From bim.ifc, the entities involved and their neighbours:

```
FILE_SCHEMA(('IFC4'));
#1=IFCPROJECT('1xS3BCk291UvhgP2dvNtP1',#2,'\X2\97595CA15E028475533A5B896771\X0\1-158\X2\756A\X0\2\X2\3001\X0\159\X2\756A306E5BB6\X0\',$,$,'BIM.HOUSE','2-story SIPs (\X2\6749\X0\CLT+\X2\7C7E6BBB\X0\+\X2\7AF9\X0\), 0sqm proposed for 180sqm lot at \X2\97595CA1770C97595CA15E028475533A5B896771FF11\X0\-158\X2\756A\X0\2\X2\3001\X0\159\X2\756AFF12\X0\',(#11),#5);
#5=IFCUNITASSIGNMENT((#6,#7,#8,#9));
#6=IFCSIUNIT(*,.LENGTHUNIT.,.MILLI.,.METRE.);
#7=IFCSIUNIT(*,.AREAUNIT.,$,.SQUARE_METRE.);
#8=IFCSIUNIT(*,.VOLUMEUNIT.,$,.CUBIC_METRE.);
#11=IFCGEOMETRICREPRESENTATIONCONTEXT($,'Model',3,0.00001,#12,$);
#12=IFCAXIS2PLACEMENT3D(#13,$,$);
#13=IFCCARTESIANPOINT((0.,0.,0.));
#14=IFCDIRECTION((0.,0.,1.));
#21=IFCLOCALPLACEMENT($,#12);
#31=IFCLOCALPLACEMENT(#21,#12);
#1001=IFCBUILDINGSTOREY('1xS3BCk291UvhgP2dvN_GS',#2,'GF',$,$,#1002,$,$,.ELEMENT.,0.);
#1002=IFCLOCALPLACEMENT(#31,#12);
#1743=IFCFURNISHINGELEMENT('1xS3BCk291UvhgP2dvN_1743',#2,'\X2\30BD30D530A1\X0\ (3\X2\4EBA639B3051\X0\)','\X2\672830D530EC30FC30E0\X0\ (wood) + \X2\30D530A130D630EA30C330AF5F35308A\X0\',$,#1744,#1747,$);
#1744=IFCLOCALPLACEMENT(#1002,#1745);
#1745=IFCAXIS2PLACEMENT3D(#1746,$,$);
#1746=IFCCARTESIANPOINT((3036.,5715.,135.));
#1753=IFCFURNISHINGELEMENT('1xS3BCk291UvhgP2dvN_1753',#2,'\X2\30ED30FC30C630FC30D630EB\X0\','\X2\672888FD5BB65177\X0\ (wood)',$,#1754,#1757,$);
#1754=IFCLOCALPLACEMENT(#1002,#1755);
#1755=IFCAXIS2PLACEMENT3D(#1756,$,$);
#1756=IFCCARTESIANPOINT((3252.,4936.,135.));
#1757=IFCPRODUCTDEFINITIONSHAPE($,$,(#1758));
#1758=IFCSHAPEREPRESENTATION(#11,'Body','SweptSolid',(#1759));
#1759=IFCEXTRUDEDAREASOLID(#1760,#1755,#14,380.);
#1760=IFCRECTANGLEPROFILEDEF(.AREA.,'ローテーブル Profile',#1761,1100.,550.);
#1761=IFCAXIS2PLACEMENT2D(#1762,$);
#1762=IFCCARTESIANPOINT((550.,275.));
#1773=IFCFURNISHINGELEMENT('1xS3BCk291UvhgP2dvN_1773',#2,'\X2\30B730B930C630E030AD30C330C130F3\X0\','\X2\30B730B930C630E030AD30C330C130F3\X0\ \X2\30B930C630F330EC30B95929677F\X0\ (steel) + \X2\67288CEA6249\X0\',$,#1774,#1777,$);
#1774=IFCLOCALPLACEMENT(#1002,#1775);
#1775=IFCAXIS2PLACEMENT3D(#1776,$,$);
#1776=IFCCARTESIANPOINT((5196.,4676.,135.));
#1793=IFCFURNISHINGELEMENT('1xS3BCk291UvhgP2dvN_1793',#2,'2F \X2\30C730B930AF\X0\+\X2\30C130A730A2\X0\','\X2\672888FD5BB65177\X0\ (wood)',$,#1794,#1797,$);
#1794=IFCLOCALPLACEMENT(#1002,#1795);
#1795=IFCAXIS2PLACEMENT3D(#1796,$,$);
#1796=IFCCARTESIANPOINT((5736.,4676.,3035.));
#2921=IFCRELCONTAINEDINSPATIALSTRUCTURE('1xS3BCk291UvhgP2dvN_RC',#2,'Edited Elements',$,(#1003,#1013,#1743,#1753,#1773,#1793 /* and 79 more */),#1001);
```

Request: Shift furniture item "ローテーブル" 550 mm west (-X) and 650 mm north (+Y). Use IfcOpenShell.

```python
import ifcopenshell
import ifcopenshell.api.geometry
import ifcopenshell.util.placement
import ifcopenshell.util.unit

model = ifcopenshell.open("bim.ifc")
unit_scale = ifcopenshell.util.unit.calculate_unit_scale(model)

item = model.by_guid("1xS3BCk291UvhgP2dvN_1753")
matrix = ifcopenshell.util.placement.get_local_placement(item.ObjectPlacement)
matrix[0, 3] -= 0.55 / unit_scale
matrix[1, 3] += 0.65 / unit_scale
ifcopenshell.api.geometry.edit_object_placement(model, product=item, matrix=matrix, is_si=False)

print(ifcopenshell.util.placement.get_local_placement(item.ObjectPlacement).round(3) + 0.0)

model.write("bim_v2.ifc")
```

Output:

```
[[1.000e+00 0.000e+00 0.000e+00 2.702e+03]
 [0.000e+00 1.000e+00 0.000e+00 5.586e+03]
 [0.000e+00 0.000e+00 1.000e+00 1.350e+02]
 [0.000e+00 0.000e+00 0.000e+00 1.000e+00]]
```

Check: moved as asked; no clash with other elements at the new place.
